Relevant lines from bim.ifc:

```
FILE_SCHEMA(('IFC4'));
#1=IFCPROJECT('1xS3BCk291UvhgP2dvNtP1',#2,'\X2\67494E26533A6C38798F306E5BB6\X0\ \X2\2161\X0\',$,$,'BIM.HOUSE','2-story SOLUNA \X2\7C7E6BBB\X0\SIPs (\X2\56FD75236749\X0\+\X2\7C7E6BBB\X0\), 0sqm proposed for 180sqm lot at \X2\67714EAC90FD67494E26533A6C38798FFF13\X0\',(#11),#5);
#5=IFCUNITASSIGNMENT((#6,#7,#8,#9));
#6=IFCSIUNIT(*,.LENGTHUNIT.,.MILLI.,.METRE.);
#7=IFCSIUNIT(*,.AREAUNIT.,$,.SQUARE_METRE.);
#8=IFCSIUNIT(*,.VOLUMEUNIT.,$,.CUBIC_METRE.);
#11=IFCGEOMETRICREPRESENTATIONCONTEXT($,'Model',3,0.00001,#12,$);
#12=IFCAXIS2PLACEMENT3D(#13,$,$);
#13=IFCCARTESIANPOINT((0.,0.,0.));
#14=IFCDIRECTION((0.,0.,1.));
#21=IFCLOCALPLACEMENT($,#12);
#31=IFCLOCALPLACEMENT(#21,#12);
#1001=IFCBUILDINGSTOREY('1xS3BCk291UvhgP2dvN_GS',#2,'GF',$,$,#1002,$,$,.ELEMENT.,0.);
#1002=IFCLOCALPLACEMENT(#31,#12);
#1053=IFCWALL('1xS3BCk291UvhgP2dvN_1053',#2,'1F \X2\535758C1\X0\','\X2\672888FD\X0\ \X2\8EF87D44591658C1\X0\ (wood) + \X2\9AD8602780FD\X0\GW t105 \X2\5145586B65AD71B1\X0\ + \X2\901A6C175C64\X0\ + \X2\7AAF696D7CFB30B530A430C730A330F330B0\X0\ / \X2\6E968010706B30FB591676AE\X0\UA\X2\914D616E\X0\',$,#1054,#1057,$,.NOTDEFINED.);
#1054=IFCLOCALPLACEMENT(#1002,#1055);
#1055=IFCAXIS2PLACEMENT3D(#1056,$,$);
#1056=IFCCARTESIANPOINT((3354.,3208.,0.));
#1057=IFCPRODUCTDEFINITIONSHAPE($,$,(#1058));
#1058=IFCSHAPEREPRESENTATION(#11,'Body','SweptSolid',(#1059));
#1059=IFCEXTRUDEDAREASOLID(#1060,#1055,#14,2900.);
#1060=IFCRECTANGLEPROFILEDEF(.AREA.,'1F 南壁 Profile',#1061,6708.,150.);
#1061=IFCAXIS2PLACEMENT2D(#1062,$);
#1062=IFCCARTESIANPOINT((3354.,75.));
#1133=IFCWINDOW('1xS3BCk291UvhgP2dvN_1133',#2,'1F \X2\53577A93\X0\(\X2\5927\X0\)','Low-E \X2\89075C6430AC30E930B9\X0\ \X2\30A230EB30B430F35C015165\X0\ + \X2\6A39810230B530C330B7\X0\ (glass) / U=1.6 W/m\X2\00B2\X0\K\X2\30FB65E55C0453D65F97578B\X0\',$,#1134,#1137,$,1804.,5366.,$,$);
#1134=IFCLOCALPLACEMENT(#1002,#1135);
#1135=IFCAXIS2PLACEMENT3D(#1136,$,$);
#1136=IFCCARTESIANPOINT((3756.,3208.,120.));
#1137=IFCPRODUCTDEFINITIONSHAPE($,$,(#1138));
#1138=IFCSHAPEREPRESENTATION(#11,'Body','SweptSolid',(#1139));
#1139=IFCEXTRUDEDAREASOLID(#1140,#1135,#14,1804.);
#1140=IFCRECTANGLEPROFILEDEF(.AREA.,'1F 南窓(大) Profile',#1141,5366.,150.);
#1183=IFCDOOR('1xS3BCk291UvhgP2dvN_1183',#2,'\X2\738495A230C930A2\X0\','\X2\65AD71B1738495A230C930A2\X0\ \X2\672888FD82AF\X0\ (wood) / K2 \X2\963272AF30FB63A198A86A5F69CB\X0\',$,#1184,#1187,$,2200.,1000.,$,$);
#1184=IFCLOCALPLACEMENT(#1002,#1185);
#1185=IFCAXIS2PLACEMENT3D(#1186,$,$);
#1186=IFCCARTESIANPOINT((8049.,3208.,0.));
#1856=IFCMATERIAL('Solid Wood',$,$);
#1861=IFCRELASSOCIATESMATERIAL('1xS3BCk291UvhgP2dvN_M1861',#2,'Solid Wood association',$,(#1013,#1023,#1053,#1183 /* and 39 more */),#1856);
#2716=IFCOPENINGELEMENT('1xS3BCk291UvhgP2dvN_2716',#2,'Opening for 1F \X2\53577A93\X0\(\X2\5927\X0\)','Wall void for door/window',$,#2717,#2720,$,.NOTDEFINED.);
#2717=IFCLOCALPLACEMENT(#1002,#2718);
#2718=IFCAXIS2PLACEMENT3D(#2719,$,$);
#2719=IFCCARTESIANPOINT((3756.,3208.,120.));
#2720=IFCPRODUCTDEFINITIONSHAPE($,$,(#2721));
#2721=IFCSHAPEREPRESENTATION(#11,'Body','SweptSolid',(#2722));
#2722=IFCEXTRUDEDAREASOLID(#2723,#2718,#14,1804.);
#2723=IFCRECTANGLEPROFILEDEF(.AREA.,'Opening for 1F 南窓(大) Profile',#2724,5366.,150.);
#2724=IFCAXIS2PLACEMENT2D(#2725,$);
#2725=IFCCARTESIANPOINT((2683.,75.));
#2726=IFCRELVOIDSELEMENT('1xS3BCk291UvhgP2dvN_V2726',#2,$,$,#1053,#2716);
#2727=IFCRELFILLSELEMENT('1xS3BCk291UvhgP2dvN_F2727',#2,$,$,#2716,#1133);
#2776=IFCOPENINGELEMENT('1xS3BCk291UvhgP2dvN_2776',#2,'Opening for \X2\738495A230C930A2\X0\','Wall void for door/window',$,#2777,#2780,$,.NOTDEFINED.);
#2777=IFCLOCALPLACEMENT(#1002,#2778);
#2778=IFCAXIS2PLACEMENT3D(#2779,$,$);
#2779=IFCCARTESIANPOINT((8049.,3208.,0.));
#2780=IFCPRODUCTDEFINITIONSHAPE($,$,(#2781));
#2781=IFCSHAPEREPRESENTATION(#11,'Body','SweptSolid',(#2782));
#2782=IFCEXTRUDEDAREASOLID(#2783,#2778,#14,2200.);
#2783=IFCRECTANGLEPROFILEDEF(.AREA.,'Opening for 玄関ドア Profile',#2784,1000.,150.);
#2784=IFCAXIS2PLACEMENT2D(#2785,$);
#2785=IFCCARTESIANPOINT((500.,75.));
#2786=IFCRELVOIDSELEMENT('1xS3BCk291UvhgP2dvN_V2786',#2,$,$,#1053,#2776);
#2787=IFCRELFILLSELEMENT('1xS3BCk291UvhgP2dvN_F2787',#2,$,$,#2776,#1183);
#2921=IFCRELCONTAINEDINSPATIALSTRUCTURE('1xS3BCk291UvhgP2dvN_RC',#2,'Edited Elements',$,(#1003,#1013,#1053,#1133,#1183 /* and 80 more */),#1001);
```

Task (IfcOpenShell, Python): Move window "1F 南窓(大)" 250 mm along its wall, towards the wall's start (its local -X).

```python
import ifcopenshell
import ifcopenshell.api.geometry
import ifcopenshell.util.placement
import ifcopenshell.util.unit

model = ifcopenshell.open("bim.ifc")
unit_scale = ifcopenshell.util.unit.calculate_unit_scale(model)

window = model.by_guid("1xS3BCk291UvhgP2dvN_1133")
opening = window.FillsVoids[0].RelatingOpeningElement
wall = opening.VoidsElements[0].RelatingBuildingElement

wall_matrix = ifcopenshell.util.placement.get_local_placement(wall.ObjectPlacement)
shift = wall_matrix[:3, 0] * -0.25 / unit_scale
before = ifcopenshell.util.placement.get_local_placement(window.ObjectPlacement)[:3, 3].copy()

# The window is not placed relative to its opening, so move both.
for product in (opening, window):
    matrix = ifcopenshell.util.placement.get_local_placement(product.ObjectPlacement)
    matrix[:3, 3] += shift
    ifcopenshell.api.geometry.edit_object_placement(model, product=product, matrix=matrix, is_si=False)

after = ifcopenshell.util.placement.get_local_placement(window.ObjectPlacement)[:3, 3]
print("window moved by", (after - before).round(3) + 0.0)

model.write("bim-out.ifc")
```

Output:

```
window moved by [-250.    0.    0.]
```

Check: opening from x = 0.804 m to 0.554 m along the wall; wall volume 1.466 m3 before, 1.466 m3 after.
